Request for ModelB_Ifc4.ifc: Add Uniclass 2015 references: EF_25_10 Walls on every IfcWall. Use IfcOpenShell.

First a look at what the model holds.

```python
import ifcopenshell

model = ifcopenshell.open("ModelB_Ifc4.ifc")
print(model.schema)
print("classifications:", [c.Name for c in model.by_type("IfcClassification")])
for ifc_class in ("IfcDoor", "IfcRoof", "IfcStair", "IfcWall", "IfcWindow"):
    print(ifc_class, len(model.by_type(ifc_class)))
```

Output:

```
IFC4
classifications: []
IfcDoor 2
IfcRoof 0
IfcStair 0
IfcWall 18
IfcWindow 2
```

```python
import ifcopenshell
import ifcopenshell.api.classification

model = ifcopenshell.open("ModelB_Ifc4.ifc")

system = ifcopenshell.api.classification.add_classification(model, classification="Uniclass 2015")

codes = {
    "IfcWall": ("EF_25_10", "Walls"),
}
for ifc_class, (code, name) in codes.items():
    products = model.by_type(ifc_class)
    ifcopenshell.api.classification.add_reference(
        model, products=products, classification=system, identification=code, name=name
    )
    print(code, len(products))

model.write("ModelB_Ifc4_updated.ifc")
```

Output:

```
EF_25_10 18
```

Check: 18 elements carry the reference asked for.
